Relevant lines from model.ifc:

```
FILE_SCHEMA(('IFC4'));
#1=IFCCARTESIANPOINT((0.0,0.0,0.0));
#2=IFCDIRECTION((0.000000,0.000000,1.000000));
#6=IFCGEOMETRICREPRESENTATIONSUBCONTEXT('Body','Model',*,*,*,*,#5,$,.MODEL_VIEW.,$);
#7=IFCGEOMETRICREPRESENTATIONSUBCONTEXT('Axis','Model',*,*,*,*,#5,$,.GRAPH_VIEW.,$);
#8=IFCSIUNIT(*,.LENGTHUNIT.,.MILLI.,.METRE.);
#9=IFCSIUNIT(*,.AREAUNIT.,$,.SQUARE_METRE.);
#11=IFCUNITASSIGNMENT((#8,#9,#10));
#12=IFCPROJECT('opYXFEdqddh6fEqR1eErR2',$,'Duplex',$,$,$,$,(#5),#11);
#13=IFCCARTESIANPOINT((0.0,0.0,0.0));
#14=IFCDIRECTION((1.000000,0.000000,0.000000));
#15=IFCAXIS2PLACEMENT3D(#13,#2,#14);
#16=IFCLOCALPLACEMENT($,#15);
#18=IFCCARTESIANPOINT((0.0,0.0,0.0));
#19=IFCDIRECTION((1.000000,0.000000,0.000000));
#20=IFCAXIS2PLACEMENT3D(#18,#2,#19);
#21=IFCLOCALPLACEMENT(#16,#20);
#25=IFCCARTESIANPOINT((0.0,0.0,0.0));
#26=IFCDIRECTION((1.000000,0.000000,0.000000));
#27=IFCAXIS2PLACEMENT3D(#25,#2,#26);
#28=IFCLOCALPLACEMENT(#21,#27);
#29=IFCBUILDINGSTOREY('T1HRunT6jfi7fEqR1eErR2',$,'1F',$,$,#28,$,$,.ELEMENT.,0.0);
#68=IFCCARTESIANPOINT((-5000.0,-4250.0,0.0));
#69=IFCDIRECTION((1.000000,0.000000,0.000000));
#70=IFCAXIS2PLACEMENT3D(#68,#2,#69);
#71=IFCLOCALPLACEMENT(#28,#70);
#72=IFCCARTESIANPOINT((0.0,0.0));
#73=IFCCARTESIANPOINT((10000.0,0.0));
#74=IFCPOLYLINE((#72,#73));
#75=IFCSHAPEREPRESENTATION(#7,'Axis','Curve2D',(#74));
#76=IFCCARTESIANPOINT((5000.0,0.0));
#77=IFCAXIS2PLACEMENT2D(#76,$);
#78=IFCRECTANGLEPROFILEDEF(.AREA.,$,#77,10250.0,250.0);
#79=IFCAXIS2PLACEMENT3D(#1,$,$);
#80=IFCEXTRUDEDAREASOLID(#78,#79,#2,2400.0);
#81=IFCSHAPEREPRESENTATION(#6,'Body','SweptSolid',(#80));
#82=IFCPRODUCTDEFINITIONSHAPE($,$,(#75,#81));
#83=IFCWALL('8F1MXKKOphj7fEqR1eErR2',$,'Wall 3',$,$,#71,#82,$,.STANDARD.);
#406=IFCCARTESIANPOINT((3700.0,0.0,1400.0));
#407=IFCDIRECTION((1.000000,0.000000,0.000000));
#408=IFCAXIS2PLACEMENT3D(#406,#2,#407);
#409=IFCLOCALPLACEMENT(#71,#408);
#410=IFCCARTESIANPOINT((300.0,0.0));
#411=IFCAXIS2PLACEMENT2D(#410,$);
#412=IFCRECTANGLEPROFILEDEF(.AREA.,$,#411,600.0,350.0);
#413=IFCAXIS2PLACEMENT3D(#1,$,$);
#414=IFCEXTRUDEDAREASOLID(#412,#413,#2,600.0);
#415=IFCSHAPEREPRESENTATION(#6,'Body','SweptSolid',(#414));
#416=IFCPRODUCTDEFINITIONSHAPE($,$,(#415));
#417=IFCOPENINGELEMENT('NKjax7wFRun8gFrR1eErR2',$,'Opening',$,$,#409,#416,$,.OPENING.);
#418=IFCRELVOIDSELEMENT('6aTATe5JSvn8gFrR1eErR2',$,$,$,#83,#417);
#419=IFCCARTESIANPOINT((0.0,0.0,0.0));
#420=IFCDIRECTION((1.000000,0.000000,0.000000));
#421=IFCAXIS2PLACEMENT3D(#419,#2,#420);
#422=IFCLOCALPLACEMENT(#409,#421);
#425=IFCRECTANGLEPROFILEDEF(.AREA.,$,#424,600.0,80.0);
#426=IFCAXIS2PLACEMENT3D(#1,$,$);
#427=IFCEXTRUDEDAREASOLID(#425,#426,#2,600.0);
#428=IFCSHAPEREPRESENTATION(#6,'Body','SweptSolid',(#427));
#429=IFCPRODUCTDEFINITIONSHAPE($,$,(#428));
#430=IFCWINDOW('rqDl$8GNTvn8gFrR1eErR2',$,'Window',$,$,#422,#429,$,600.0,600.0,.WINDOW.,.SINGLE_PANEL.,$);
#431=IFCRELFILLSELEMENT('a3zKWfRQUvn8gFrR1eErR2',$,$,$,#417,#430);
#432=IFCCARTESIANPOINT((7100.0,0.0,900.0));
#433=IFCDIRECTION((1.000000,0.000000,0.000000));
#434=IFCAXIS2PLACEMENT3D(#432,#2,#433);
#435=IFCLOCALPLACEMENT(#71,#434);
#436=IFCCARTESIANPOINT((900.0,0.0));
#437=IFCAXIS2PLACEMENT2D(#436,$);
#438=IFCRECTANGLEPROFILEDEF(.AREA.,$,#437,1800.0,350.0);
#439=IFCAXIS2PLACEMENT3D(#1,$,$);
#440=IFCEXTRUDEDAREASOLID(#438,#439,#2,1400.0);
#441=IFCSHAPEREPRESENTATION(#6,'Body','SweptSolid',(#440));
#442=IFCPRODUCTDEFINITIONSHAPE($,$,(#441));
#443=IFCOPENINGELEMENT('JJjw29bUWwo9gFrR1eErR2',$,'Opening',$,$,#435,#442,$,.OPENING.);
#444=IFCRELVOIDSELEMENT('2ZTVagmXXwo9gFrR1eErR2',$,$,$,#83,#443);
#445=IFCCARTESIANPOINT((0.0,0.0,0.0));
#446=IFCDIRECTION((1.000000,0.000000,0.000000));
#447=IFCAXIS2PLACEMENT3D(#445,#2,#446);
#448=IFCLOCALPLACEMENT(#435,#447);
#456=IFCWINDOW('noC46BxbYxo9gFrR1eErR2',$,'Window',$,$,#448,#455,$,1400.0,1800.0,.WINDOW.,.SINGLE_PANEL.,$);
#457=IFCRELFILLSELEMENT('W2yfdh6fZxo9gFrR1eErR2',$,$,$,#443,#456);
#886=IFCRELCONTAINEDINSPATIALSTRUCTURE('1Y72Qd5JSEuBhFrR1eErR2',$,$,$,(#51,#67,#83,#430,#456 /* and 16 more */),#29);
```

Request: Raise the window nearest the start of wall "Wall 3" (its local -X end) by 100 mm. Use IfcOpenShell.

```python
import numpy as np
import ifcopenshell
import ifcopenshell.api.geometry
import ifcopenshell.util.placement
import ifcopenshell.util.unit

model = ifcopenshell.open("model.ifc")
unit_scale = ifcopenshell.util.unit.calculate_unit_scale(model)

window = model.by_guid("rqDl$8GNTvn8gFrR1eErR2")
opening = window.FillsVoids[0].RelatingOpeningElement
dz = 100.0

shift = np.array([0.0, 0.0, dz])
# The window is placed relative to its opening, so it follows when the opening moves.
matrix = ifcopenshell.util.placement.get_local_placement(opening.ObjectPlacement)
matrix[:3, 3] += shift
ifcopenshell.api.geometry.edit_object_placement(
    model, product=opening, matrix=matrix, is_si=False, should_transform_children=True
)

print(f"moved by {dz * unit_scale:+.3f} m")

model.write("model_v2.ifc")
```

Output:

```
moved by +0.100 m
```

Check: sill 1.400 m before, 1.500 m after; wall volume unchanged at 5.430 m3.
